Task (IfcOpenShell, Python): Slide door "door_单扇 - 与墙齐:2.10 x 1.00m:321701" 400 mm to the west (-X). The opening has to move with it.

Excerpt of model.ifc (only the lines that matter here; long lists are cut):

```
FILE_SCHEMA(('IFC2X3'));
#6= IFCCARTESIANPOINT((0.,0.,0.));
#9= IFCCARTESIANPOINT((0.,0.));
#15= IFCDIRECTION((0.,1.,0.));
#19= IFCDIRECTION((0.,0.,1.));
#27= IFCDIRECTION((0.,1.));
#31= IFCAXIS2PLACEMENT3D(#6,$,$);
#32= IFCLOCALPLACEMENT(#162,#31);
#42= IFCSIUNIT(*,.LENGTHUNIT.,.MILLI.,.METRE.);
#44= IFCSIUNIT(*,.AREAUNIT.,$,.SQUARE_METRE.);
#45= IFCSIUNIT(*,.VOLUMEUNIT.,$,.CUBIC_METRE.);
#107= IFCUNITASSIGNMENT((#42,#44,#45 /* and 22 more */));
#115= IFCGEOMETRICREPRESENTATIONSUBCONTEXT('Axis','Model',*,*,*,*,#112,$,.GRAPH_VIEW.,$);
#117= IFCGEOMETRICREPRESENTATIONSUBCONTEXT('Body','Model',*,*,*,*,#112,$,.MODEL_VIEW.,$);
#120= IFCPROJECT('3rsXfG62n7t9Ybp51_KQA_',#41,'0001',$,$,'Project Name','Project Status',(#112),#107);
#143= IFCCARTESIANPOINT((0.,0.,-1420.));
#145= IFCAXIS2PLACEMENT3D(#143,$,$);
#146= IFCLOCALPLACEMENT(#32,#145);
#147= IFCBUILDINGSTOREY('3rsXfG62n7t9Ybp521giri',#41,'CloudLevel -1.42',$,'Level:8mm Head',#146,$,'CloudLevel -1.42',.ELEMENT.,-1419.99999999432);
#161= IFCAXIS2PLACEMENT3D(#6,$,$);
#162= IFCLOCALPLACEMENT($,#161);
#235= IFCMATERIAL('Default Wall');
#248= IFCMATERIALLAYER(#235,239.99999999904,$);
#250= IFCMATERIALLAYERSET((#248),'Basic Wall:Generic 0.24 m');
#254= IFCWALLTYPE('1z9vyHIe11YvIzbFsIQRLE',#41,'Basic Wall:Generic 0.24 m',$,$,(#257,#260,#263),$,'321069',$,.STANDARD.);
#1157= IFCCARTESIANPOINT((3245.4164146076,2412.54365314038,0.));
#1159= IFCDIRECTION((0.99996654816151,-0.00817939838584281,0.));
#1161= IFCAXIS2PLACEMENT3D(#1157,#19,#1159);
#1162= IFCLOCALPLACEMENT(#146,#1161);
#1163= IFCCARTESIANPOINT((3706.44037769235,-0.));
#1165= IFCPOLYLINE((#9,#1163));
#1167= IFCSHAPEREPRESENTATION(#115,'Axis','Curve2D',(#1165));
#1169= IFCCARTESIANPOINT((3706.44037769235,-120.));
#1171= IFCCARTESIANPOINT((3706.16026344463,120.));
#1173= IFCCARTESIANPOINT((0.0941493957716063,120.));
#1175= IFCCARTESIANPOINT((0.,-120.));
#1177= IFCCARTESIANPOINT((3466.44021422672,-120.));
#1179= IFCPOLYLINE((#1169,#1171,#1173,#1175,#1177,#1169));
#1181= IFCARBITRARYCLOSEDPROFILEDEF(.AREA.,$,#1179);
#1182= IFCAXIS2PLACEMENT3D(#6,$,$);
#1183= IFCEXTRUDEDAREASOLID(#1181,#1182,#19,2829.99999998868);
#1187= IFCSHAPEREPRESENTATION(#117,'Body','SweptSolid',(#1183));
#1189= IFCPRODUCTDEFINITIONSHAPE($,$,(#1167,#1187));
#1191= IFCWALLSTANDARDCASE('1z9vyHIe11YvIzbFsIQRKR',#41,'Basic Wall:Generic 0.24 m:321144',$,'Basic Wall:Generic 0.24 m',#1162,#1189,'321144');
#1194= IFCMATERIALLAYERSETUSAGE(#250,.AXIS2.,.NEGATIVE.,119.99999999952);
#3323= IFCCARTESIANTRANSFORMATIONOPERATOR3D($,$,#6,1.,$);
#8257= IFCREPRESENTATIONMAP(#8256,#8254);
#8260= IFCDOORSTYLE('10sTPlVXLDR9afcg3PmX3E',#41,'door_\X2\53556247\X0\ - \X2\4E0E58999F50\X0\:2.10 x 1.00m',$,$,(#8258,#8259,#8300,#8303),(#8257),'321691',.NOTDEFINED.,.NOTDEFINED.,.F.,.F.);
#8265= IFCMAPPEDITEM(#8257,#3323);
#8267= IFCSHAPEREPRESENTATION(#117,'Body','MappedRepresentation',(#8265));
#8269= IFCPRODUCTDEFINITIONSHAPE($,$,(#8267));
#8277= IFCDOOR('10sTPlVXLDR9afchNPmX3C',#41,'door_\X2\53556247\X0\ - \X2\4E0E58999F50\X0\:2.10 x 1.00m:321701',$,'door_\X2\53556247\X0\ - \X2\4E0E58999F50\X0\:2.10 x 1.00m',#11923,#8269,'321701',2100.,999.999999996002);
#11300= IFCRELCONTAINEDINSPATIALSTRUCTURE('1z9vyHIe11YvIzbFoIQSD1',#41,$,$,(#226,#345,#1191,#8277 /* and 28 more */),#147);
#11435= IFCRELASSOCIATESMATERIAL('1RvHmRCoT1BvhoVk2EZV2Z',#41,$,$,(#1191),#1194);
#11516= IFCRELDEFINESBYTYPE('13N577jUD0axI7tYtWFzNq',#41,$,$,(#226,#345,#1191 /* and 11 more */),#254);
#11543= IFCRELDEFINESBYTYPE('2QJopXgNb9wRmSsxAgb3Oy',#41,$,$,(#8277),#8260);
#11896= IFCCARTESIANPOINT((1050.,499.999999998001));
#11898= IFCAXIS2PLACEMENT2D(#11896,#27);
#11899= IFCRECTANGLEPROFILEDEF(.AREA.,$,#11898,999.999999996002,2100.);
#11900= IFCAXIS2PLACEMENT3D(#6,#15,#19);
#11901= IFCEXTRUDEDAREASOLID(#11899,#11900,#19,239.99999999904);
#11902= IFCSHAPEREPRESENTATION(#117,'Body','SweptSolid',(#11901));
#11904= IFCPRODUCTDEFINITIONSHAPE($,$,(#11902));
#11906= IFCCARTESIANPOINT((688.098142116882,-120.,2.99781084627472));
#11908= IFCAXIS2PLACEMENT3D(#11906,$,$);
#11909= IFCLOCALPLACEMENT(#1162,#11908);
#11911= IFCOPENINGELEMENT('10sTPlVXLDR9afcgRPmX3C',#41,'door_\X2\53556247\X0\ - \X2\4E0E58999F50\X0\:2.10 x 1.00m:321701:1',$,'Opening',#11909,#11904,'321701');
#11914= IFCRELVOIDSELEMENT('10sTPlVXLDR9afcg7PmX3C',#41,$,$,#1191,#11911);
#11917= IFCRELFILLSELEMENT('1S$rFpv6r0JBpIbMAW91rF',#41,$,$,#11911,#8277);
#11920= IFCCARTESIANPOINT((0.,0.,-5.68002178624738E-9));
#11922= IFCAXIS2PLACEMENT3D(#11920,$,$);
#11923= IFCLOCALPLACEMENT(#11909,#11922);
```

```python
import ifcopenshell
import ifcopenshell.api.geometry
import ifcopenshell.util.placement
import ifcopenshell.util.unit

model = ifcopenshell.open("model.ifc")
unit_scale = ifcopenshell.util.unit.calculate_unit_scale(model)

door = model.by_guid("10sTPlVXLDR9afchNPmX3C")
opening = door.FillsVoids[0].RelatingOpeningElement
wall = opening.VoidsElements[0].RelatingBuildingElement

wall_matrix = ifcopenshell.util.placement.get_local_placement(wall.ObjectPlacement)
shift = wall_matrix[:3, 0] * -0.4 / unit_scale
before = ifcopenshell.util.placement.get_local_placement(door.ObjectPlacement)[:3, 3].copy()

# The door is placed relative to its opening, so it follows when the opening moves.
matrix = ifcopenshell.util.placement.get_local_placement(opening.ObjectPlacement)
matrix[:3, 3] += shift
ifcopenshell.api.geometry.edit_object_placement(
    model, product=opening, matrix=matrix, is_si=False, should_transform_children=True
)

after = ifcopenshell.util.placement.get_local_placement(door.ObjectPlacement)[:3, 3]
print("door moved by", (after - before).round(3) + 0.0)

model.write("model_edited.ifc")
```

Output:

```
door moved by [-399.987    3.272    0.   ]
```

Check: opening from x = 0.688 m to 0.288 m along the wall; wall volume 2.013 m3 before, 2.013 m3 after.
